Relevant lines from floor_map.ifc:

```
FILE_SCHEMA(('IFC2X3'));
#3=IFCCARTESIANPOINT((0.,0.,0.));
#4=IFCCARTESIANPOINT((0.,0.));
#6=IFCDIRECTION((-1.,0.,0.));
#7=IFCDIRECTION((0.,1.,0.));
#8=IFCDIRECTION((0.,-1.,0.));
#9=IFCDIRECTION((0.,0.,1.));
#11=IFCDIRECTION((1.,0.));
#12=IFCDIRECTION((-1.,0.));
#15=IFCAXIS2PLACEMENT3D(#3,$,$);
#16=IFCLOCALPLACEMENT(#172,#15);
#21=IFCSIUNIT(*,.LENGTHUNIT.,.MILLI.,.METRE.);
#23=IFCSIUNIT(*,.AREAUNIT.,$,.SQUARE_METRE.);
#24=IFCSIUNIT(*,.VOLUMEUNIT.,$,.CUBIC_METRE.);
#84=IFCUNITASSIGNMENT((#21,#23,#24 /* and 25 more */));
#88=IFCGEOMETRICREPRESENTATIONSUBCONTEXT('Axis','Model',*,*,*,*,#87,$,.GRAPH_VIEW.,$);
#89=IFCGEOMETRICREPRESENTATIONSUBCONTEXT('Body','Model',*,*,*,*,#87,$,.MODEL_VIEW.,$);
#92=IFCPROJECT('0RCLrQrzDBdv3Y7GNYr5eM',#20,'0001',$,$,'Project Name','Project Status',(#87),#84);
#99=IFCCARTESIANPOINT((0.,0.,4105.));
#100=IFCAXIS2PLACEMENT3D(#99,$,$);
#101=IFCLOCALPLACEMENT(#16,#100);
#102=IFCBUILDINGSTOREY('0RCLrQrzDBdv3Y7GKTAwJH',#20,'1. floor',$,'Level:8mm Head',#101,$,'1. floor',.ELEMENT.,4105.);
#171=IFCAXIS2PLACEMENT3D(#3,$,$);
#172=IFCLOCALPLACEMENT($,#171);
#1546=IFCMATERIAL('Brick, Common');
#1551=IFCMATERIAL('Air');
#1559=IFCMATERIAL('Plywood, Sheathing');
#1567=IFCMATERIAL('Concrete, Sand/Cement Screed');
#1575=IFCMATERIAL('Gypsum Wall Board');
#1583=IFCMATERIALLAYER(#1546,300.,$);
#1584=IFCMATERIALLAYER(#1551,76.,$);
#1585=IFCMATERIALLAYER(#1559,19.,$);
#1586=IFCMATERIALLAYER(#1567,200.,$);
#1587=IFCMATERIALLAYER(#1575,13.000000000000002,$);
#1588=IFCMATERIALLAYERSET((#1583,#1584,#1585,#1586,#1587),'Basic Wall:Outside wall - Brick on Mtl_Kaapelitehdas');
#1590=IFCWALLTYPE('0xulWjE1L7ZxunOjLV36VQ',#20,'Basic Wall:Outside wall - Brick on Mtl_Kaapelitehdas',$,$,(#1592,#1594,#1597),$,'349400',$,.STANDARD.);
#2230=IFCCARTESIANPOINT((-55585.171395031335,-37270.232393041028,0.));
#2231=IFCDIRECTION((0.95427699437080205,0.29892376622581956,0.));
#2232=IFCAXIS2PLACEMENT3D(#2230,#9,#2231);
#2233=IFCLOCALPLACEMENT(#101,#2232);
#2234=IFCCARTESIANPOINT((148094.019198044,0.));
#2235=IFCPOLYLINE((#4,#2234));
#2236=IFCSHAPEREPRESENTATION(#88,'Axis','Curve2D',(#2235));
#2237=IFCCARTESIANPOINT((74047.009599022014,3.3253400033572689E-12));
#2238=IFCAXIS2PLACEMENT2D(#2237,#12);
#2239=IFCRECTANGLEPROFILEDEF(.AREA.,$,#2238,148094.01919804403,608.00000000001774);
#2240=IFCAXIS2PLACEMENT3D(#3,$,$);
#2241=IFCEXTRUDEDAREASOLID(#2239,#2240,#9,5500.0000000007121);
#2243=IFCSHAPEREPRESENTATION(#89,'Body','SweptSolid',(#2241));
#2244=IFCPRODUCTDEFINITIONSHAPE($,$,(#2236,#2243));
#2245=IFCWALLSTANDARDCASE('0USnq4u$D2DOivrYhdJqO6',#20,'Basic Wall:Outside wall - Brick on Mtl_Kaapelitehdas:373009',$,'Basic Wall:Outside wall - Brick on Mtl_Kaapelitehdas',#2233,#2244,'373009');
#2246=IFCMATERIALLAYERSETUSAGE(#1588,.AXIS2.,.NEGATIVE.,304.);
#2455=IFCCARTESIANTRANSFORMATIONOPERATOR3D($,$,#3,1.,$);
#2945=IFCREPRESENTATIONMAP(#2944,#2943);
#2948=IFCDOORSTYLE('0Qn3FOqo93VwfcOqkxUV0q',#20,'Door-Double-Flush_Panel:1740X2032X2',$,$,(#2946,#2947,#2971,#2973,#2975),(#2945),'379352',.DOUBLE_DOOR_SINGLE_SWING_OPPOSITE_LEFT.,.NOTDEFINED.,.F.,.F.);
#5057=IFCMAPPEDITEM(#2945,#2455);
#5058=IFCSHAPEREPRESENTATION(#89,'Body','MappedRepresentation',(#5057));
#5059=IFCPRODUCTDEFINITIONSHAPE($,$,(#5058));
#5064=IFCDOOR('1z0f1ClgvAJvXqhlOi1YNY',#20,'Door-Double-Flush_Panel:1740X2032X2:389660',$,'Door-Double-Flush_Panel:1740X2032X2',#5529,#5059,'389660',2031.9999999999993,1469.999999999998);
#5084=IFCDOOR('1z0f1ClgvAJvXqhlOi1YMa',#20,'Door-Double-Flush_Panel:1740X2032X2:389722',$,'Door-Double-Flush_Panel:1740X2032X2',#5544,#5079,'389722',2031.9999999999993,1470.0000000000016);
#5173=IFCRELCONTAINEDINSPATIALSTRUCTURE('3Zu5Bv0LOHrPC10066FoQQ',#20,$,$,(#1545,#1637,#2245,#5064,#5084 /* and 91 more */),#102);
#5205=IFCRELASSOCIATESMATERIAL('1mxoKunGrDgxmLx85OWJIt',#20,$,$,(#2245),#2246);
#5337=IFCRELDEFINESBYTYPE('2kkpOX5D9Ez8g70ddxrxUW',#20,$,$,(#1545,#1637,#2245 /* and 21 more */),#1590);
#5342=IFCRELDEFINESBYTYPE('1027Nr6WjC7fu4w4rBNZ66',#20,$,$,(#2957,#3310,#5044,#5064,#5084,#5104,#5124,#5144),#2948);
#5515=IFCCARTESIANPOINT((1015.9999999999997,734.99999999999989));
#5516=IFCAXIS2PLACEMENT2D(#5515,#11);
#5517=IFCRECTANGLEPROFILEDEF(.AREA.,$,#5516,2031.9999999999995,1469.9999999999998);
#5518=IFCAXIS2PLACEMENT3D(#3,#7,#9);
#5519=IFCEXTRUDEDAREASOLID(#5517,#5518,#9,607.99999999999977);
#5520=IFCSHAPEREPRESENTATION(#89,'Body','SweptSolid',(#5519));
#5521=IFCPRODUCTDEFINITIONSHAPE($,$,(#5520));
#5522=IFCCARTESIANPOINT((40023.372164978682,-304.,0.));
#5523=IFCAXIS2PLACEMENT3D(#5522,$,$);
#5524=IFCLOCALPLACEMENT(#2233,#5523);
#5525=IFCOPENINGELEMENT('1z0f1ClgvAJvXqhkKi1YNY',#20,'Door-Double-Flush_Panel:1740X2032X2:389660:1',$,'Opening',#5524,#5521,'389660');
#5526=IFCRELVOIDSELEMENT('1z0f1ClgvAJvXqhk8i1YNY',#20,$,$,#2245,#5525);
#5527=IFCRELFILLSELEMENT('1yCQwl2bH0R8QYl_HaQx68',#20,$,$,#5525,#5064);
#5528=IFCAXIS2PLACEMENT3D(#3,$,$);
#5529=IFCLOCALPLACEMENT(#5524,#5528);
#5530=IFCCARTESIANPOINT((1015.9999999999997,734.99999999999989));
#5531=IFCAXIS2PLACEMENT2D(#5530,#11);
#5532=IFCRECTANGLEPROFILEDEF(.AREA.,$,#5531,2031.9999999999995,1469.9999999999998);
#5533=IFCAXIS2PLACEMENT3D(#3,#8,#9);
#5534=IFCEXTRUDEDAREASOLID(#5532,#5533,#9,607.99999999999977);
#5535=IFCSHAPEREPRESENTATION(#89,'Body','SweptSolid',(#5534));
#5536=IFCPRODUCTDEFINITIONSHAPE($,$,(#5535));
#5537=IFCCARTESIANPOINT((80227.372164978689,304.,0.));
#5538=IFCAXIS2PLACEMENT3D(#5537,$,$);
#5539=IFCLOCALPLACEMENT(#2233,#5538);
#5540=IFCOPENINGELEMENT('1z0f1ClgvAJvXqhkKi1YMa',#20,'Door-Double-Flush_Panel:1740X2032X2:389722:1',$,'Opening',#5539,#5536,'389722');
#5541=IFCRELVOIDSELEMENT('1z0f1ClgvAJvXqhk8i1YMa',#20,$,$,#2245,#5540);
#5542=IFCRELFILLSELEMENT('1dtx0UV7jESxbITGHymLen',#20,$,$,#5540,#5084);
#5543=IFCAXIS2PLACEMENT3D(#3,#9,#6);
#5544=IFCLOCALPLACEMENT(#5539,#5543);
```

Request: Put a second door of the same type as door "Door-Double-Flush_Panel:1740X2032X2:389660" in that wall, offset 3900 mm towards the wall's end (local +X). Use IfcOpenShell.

```python
import ifcopenshell
import ifcopenshell.api.feature
import ifcopenshell.api.geometry
import ifcopenshell.api.root
import ifcopenshell.geom
import ifcopenshell.util.element
import ifcopenshell.util.placement
import ifcopenshell.util.shape

model = ifcopenshell.open("floor_map.ifc")
settings = ifcopenshell.geom.settings()


def volume(element):
    """Net volume in cubic metres, openings subtracted."""
    shape = ifcopenshell.geom.create_shape(settings, element)
    return ifcopenshell.util.shape.get_volume(shape.geometry)


def reuse_history(source, copy):
    """copy_class also copies each property set's owner history, people and application; keep the originals."""
    for rel in copy.IsDefinedBy:
        if rel.is_a("IfcRelDefinesByProperties") and (history := rel.RelatingPropertyDefinition.OwnerHistory):
            rel.RelatingPropertyDefinition.OwnerHistory = source.OwnerHistory
            ifcopenshell.util.element.remove_deep2(model, history)


door = model.by_guid("1z0f1ClgvAJvXqhlOi1YNY")
opening = door.FillsVoids[0].RelatingOpeningElement
wall = opening.VoidsElements[0].RelatingBuildingElement
before = volume(wall)
shift = ifcopenshell.util.placement.get_local_placement(wall.ObjectPlacement)[:3, 0] * 3900.0

# copy_class copies the void relationship, type, container and properties, but no geometry.
new_opening = ifcopenshell.api.root.copy_class(model, product=opening)
new_opening.Representation = ifcopenshell.util.element.copy_deep(
    model, opening.Representation, exclude=["IfcGeometricRepresentationContext", "IfcRepresentationMap"]
)
new_opening.Name = "Door-Double-Flush_Panel:1740X2032X2"
new_opening.Tag = None
new_door = ifcopenshell.api.root.copy_class(model, product=door)
new_door.Representation = ifcopenshell.util.element.copy_deep(
    model, door.Representation, exclude=["IfcGeometricRepresentationContext", "IfcRepresentationMap"]
)
new_door.Name = "Door-Double-Flush_Panel:1740X2032X2"
new_door.Tag = None
reuse_history(door, new_door)
fills = ifcopenshell.api.feature.add_filling(model, opening=new_opening, element=new_door)
fills.OwnerHistory = new_door.OwnerHistory  # required in IFC2X3

for old, new in ((opening, new_opening), (door, new_door)):
    matrix = ifcopenshell.util.placement.get_local_placement(old.ObjectPlacement)
    matrix[:3, 3] += shift
    ifcopenshell.api.geometry.edit_object_placement(model, product=new, matrix=matrix, is_si=False)

after = volume(wall)

print(f"wall volume {before:.3f} -> {after:.3f} m3")

model.write("floor_map-out.ifc")
```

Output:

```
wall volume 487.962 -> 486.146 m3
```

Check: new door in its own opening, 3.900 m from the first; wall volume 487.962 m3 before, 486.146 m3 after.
